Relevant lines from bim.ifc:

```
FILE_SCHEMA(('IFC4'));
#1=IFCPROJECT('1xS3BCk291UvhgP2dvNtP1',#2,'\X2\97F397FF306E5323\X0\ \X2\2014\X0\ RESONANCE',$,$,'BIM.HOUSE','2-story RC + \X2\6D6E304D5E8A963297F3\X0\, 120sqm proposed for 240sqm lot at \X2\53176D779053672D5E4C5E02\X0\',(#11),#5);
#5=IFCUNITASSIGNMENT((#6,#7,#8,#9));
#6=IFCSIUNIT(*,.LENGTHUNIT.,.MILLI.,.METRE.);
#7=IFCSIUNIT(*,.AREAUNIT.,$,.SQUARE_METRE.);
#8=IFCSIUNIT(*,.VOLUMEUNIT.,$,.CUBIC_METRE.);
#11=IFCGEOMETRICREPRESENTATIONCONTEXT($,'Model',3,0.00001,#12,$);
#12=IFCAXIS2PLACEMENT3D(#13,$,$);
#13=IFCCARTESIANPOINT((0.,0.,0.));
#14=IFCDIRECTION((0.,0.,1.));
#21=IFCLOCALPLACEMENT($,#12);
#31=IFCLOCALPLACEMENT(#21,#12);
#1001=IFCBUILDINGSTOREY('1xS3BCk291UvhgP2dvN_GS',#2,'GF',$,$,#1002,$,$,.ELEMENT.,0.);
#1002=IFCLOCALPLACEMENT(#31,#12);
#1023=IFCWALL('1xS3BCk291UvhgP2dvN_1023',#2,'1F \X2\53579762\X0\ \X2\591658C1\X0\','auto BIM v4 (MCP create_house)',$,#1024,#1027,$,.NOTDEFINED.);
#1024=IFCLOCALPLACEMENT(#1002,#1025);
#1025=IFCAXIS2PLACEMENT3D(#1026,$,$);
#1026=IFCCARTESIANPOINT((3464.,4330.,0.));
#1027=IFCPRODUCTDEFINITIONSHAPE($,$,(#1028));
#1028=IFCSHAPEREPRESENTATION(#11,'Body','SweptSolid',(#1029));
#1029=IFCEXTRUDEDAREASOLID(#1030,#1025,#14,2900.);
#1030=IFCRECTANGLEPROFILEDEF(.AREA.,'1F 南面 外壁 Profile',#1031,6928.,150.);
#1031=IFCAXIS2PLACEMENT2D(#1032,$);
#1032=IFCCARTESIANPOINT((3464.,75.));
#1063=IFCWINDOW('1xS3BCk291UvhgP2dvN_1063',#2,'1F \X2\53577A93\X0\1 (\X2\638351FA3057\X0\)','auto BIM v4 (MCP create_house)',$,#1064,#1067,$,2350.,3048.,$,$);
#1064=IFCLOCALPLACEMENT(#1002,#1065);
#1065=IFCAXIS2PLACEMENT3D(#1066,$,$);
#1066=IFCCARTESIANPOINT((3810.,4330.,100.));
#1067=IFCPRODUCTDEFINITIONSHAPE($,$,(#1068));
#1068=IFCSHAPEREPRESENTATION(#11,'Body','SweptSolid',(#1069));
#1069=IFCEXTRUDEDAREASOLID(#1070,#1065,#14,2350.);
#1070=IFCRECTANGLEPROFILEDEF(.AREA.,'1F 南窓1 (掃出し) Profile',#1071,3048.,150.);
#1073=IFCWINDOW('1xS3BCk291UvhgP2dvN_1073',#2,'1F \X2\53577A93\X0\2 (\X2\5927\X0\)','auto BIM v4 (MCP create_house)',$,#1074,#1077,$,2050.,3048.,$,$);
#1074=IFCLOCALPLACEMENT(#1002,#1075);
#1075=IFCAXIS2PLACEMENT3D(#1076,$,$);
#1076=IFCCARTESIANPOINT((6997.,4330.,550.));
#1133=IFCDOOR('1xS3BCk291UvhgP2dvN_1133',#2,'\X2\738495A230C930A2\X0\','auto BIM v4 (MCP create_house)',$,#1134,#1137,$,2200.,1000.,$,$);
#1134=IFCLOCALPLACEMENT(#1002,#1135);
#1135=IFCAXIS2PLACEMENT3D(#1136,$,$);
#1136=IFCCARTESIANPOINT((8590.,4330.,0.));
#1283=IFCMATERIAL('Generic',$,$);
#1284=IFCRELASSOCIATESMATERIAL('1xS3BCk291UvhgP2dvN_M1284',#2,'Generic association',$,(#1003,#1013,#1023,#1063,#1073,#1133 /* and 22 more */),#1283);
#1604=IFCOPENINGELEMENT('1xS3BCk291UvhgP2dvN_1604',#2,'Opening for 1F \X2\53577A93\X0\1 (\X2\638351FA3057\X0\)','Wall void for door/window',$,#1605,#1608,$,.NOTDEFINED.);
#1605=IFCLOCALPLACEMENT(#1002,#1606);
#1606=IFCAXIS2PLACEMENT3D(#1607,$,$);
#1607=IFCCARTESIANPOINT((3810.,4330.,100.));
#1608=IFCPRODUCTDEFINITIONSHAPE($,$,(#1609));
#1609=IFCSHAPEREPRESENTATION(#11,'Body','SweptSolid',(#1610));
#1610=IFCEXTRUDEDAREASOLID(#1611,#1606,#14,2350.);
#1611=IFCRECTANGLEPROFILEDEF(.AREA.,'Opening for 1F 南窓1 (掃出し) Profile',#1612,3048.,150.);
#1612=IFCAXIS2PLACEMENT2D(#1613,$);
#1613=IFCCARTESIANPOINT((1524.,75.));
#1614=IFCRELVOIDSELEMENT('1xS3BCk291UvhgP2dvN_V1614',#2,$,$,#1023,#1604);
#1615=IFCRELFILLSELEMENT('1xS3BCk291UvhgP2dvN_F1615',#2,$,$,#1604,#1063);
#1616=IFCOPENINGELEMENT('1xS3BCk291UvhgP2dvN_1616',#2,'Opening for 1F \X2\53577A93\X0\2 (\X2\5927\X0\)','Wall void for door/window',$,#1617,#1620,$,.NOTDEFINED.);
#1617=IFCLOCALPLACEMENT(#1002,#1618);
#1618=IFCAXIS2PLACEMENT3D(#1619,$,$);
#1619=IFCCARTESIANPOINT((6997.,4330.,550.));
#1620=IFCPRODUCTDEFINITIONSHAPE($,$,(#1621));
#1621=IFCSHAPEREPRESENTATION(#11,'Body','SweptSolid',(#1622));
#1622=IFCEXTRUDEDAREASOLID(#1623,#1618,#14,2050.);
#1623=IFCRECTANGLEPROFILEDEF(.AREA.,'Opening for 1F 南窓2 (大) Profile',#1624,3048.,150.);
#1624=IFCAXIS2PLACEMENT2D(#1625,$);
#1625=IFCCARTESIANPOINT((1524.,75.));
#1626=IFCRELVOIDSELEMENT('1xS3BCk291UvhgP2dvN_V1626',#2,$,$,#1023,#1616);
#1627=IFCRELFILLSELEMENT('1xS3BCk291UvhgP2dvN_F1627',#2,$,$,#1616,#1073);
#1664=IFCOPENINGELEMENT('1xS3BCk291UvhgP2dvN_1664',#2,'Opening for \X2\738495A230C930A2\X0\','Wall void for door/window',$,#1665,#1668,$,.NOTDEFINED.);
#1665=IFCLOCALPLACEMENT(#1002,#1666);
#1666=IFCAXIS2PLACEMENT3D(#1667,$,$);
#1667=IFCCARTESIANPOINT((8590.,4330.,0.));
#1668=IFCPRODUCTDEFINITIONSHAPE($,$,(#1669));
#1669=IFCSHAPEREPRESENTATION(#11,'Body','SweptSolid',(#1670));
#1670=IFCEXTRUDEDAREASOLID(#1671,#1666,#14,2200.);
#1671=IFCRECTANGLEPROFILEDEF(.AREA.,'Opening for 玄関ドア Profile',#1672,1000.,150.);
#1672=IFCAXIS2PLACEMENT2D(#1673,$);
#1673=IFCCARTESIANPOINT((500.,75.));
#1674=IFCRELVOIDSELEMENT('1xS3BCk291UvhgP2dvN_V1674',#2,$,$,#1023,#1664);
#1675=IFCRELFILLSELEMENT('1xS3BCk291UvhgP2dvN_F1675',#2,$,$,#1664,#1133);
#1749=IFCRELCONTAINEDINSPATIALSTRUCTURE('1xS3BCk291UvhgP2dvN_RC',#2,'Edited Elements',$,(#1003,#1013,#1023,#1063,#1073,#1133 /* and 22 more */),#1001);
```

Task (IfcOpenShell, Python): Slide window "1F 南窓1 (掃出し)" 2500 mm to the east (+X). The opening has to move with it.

```python
import ifcopenshell
import ifcopenshell.api.geometry
import ifcopenshell.util.placement
import ifcopenshell.util.unit

model = ifcopenshell.open("bim.ifc")
unit_scale = ifcopenshell.util.unit.calculate_unit_scale(model)

window = model.by_id(1063)
opening = window.FillsVoids[0].RelatingOpeningElement
wall = opening.VoidsElements[0].RelatingBuildingElement

wall_matrix = ifcopenshell.util.placement.get_local_placement(wall.ObjectPlacement)
shift = wall_matrix[:3, 0] * 2.5 / unit_scale
before = ifcopenshell.util.placement.get_local_placement(window.ObjectPlacement)[:3, 3].copy()

# The window is not placed relative to its opening, so move both.
for product in (opening, window):
    matrix = ifcopenshell.util.placement.get_local_placement(product.ObjectPlacement)
    matrix[:3, 3] += shift
    ifcopenshell.api.geometry.edit_object_placement(model, product=product, matrix=matrix, is_si=False)

after = ifcopenshell.util.placement.get_local_placement(window.ObjectPlacement)[:3, 3]
print("window moved by", (after - before).round(3) + 0.0)

model.write("bim_edited.ifc")
```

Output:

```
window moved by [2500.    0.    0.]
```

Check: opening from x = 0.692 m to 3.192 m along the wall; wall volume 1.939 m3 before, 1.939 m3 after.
